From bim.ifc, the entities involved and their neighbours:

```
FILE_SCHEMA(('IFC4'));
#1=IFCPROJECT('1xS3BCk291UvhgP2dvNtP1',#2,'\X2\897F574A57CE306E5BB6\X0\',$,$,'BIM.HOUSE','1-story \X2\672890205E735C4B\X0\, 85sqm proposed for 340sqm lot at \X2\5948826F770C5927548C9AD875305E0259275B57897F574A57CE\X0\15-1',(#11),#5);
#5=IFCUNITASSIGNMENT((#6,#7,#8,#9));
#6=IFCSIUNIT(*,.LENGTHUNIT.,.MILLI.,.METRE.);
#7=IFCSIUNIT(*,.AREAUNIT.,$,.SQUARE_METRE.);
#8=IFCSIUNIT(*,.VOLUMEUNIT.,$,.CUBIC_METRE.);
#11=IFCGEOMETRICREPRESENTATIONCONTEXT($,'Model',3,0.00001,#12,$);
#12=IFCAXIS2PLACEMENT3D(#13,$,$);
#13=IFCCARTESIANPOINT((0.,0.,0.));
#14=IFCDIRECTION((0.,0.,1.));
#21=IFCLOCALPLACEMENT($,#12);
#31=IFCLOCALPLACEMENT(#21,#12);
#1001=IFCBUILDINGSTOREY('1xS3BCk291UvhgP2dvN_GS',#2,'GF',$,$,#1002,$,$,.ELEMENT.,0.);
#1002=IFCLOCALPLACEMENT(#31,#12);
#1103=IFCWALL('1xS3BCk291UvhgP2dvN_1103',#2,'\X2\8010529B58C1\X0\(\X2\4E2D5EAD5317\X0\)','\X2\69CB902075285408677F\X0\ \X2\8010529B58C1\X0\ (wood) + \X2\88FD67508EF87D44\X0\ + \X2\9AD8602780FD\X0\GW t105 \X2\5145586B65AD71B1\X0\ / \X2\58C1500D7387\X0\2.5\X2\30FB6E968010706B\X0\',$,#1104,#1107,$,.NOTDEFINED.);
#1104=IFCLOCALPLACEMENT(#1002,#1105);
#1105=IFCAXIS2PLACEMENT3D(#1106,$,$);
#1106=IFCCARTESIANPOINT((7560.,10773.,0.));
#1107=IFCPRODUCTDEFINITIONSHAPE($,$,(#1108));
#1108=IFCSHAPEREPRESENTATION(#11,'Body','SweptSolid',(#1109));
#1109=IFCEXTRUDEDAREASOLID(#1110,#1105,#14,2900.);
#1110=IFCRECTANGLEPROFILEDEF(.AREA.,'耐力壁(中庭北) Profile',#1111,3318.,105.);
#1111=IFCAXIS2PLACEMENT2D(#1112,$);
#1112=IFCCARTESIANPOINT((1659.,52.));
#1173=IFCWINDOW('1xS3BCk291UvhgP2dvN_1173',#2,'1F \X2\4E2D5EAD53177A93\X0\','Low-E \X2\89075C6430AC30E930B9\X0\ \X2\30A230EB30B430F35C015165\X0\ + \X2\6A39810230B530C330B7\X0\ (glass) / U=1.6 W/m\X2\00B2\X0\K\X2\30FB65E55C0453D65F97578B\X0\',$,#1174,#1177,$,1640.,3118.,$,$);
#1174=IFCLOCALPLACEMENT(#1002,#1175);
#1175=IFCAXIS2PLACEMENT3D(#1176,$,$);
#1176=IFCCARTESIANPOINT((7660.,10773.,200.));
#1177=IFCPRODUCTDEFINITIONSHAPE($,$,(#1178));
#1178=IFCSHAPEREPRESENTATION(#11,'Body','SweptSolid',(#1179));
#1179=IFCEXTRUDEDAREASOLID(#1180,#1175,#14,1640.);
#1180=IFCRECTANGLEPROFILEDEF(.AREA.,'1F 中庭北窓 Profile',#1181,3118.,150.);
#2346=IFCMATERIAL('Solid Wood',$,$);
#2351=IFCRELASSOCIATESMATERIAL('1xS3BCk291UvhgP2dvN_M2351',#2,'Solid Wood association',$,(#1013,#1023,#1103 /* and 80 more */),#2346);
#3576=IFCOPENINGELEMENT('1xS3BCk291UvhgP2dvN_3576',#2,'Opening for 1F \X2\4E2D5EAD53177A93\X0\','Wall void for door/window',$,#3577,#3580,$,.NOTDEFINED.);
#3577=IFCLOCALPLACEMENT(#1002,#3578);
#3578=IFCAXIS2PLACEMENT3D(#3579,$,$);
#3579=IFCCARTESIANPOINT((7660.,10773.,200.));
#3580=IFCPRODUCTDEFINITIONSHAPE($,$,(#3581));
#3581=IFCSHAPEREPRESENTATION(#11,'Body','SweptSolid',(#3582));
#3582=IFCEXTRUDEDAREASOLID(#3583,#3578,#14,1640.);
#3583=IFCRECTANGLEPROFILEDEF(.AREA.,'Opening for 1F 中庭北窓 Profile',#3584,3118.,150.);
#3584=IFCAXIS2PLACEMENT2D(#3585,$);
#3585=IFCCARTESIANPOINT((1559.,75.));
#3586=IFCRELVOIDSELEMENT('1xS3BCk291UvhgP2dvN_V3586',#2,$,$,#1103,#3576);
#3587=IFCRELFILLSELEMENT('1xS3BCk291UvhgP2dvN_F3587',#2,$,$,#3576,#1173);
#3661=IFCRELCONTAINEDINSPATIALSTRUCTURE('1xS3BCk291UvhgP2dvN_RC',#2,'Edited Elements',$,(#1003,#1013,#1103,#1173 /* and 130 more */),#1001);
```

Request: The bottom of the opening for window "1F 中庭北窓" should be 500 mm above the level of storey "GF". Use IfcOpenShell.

```python
import numpy as np
import ifcopenshell
import ifcopenshell.api.geometry
import ifcopenshell.geom
import ifcopenshell.util.element
import ifcopenshell.util.placement
import ifcopenshell.util.shape
import ifcopenshell.util.unit

model = ifcopenshell.open("bim.ifc")
unit_scale = ifcopenshell.util.unit.calculate_unit_scale(model)

window = model.by_guid("1xS3BCk291UvhgP2dvN_1173")
opening = window.FillsVoids[0].RelatingOpeningElement
storey = ifcopenshell.util.element.get_container(window, ifc_class="IfcBuildingStorey")
level = ifcopenshell.util.placement.get_local_placement(storey.ObjectPlacement)[2, 3]

# The opening's origin need not be at the sill, so measure its lowest point.
shape = ifcopenshell.geom.create_shape(ifcopenshell.geom.settings(), opening)
bottom = ifcopenshell.util.shape.get_shape_bottom_elevation(shape, shape.geometry) / unit_scale
dz = level + 0.5 / unit_scale - bottom

shift = np.array([0.0, 0.0, dz])
# The window is not placed relative to its opening, so move both.
for product in (opening, window):
    matrix = ifcopenshell.util.placement.get_local_placement(product.ObjectPlacement)
    matrix[:3, 3] += shift
    ifcopenshell.api.geometry.edit_object_placement(model, product=product, matrix=matrix, is_si=False)

print(f"moved by {dz * unit_scale:+.3f} m")

model.write("bim_v2.ifc")
```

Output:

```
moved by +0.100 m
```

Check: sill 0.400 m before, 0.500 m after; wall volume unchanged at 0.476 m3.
